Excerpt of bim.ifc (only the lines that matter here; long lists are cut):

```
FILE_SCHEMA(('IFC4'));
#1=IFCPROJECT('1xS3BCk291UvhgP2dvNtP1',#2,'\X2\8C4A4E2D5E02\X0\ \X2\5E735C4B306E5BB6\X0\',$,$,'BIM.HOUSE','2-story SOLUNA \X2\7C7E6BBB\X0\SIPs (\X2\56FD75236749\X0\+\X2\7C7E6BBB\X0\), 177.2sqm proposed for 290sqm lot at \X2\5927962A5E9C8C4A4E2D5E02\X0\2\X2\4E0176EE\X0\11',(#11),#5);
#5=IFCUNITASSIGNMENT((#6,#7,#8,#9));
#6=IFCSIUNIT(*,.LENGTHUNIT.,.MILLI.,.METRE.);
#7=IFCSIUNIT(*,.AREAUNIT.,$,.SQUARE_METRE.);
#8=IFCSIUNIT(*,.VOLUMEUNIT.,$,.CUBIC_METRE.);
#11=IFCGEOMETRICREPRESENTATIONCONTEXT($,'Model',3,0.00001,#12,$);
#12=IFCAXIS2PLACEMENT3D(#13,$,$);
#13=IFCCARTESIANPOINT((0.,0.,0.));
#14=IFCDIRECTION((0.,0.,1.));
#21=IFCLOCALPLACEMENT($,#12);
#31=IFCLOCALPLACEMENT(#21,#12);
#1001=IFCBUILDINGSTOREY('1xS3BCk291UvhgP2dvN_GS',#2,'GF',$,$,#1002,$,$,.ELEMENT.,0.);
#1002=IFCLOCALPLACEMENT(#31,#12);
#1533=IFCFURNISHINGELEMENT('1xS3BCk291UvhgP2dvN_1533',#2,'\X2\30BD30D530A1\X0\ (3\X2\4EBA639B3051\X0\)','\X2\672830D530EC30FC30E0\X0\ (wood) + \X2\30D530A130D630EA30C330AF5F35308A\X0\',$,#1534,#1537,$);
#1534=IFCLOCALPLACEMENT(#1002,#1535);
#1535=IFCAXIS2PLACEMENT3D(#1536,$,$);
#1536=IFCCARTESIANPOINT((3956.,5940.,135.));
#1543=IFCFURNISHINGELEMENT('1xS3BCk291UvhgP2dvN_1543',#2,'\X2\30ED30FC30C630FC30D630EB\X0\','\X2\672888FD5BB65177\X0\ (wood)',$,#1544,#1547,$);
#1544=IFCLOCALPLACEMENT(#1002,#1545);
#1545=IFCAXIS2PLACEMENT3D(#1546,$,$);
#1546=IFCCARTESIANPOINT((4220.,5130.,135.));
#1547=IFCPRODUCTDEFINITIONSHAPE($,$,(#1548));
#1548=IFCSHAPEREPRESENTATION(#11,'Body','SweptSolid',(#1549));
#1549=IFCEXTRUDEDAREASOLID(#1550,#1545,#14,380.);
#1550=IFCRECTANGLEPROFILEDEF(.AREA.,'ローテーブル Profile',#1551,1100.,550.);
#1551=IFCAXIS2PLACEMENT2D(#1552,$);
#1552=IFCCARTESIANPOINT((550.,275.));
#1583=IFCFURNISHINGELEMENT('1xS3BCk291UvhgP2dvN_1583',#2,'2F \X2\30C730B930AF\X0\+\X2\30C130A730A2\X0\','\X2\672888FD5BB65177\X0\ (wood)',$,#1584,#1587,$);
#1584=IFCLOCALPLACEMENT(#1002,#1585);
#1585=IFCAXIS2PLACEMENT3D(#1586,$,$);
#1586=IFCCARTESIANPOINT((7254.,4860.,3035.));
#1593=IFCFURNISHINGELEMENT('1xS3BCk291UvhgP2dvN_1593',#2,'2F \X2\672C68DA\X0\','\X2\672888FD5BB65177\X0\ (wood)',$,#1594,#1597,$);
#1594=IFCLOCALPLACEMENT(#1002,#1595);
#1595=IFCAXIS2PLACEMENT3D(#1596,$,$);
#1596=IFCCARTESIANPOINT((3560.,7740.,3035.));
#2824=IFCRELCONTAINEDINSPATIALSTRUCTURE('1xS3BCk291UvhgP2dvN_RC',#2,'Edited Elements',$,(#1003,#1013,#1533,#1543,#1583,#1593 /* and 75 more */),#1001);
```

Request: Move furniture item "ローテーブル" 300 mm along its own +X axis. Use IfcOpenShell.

```python
import ifcopenshell
import ifcopenshell.api.geometry
import ifcopenshell.util.placement

model = ifcopenshell.open("bim.ifc")

item = model.by_guid("1xS3BCk291UvhgP2dvN_1543")
matrix = ifcopenshell.util.placement.get_local_placement(item.ObjectPlacement)
matrix[:3, 3] += matrix[:3, 0] * 300.0
ifcopenshell.api.geometry.edit_object_placement(model, product=item, matrix=matrix, is_si=False)

print(ifcopenshell.util.placement.get_local_placement(item.ObjectPlacement).round(3) + 0.0)

model.write("bim-out.ifc")
```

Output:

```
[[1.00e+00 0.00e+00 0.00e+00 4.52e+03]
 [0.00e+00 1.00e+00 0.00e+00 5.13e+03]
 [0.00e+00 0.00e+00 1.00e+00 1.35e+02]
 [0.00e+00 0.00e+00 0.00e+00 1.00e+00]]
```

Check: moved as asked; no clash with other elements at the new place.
